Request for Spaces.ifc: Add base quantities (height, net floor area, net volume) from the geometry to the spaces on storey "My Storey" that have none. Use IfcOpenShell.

First a look at what the model holds.

```python
import ifcopenshell
import ifcopenshell.util.element
import ifcopenshell.util.unit

model = ifcopenshell.open("Spaces.ifc")
print(model.schema)
for unit_type in ("LENGTHUNIT", "AREAUNIT", "VOLUMEUNIT"):
    print(unit_type, ifcopenshell.util.unit.calculate_unit_scale(model, unit_type))
storey = next(s for s in model.by_type("IfcBuildingStorey") if s.Name == "My Storey")
spaces = [e for e in ifcopenshell.util.element.get_decomposition(storey) if e.is_a("IfcSpace")]
for e in sorted(spaces, key=lambda e: e.id()):
    print(e.id(), e.is_a(), e.Name, list(ifcopenshell.util.element.get_psets(e, qtos_only=True)), sep=" | ")
```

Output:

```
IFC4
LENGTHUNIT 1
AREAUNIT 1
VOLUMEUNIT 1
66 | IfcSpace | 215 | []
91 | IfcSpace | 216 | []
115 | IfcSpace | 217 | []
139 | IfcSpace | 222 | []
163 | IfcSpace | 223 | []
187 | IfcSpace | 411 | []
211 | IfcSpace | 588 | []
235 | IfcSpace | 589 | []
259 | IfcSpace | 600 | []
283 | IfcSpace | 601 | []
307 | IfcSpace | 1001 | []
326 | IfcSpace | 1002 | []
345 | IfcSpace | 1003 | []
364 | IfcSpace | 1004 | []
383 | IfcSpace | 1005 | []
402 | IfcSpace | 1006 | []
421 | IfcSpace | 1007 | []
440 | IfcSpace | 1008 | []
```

```python
import ifcopenshell
import ifcopenshell.api.pset
import ifcopenshell.geom
import ifcopenshell.util.element
import ifcopenshell.util.shape
import ifcopenshell.util.unit

model = ifcopenshell.open("Spaces.ifc")
unit_scale = ifcopenshell.util.unit.calculate_unit_scale(model)
area_scale = ifcopenshell.util.unit.calculate_unit_scale(model, "AREAUNIT")
volume_scale = ifcopenshell.util.unit.calculate_unit_scale(model, "VOLUMEUNIT")
settings = ifcopenshell.geom.settings()

storey = next(s for s in model.by_type("IfcBuildingStorey") if s.Name == "My Storey")
spaces = [e for e in ifcopenshell.util.element.get_decomposition(storey) if e.is_a("IfcSpace")]

for e in sorted(spaces, key=lambda e: e.id()):
    if ifcopenshell.util.element.get_psets(e, qtos_only=True, should_inherit=False):
        continue
    # Geometry comes back in metres, in the element's own axes.
    shape = ifcopenshell.geom.create_shape(settings, e)
    values = {
        "Height": ifcopenshell.util.shape.get_z(shape.geometry) / unit_scale,
        "NetFloorArea": ifcopenshell.util.shape.get_footprint_area(shape.geometry) / area_scale,
        "NetVolume": ifcopenshell.util.shape.get_volume(shape.geometry) / volume_scale,
    }
    qto = ifcopenshell.api.pset.add_qto(model, product=e, name="Qto_SpaceBaseQuantities")
    ifcopenshell.api.pset.edit_qto(model, qto=qto, properties=values)
    print(e.id(), {k: round(v, 3) for k, v in values.items()})

model.write("Spaces_updated.ifc")
```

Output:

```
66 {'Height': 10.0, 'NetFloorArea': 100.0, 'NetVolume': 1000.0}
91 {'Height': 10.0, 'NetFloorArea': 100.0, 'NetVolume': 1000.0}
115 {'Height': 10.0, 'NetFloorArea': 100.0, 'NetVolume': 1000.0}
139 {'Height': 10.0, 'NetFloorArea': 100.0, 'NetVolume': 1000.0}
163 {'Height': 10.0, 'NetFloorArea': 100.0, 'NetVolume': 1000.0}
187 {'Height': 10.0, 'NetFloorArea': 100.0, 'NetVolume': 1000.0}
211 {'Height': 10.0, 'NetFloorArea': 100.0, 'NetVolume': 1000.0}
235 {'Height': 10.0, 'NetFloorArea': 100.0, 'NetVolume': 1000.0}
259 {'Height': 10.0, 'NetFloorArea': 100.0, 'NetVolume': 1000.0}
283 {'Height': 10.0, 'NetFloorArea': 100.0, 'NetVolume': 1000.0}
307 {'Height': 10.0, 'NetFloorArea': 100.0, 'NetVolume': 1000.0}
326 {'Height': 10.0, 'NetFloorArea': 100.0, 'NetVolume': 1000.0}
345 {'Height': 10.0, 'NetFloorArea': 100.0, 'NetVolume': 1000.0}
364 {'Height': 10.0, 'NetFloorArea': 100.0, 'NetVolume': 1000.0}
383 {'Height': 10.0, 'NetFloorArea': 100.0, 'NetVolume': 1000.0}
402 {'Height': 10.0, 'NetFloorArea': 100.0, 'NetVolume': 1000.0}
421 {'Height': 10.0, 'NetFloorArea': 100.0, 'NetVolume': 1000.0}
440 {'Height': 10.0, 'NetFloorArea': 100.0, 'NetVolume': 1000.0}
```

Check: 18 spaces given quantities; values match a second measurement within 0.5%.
